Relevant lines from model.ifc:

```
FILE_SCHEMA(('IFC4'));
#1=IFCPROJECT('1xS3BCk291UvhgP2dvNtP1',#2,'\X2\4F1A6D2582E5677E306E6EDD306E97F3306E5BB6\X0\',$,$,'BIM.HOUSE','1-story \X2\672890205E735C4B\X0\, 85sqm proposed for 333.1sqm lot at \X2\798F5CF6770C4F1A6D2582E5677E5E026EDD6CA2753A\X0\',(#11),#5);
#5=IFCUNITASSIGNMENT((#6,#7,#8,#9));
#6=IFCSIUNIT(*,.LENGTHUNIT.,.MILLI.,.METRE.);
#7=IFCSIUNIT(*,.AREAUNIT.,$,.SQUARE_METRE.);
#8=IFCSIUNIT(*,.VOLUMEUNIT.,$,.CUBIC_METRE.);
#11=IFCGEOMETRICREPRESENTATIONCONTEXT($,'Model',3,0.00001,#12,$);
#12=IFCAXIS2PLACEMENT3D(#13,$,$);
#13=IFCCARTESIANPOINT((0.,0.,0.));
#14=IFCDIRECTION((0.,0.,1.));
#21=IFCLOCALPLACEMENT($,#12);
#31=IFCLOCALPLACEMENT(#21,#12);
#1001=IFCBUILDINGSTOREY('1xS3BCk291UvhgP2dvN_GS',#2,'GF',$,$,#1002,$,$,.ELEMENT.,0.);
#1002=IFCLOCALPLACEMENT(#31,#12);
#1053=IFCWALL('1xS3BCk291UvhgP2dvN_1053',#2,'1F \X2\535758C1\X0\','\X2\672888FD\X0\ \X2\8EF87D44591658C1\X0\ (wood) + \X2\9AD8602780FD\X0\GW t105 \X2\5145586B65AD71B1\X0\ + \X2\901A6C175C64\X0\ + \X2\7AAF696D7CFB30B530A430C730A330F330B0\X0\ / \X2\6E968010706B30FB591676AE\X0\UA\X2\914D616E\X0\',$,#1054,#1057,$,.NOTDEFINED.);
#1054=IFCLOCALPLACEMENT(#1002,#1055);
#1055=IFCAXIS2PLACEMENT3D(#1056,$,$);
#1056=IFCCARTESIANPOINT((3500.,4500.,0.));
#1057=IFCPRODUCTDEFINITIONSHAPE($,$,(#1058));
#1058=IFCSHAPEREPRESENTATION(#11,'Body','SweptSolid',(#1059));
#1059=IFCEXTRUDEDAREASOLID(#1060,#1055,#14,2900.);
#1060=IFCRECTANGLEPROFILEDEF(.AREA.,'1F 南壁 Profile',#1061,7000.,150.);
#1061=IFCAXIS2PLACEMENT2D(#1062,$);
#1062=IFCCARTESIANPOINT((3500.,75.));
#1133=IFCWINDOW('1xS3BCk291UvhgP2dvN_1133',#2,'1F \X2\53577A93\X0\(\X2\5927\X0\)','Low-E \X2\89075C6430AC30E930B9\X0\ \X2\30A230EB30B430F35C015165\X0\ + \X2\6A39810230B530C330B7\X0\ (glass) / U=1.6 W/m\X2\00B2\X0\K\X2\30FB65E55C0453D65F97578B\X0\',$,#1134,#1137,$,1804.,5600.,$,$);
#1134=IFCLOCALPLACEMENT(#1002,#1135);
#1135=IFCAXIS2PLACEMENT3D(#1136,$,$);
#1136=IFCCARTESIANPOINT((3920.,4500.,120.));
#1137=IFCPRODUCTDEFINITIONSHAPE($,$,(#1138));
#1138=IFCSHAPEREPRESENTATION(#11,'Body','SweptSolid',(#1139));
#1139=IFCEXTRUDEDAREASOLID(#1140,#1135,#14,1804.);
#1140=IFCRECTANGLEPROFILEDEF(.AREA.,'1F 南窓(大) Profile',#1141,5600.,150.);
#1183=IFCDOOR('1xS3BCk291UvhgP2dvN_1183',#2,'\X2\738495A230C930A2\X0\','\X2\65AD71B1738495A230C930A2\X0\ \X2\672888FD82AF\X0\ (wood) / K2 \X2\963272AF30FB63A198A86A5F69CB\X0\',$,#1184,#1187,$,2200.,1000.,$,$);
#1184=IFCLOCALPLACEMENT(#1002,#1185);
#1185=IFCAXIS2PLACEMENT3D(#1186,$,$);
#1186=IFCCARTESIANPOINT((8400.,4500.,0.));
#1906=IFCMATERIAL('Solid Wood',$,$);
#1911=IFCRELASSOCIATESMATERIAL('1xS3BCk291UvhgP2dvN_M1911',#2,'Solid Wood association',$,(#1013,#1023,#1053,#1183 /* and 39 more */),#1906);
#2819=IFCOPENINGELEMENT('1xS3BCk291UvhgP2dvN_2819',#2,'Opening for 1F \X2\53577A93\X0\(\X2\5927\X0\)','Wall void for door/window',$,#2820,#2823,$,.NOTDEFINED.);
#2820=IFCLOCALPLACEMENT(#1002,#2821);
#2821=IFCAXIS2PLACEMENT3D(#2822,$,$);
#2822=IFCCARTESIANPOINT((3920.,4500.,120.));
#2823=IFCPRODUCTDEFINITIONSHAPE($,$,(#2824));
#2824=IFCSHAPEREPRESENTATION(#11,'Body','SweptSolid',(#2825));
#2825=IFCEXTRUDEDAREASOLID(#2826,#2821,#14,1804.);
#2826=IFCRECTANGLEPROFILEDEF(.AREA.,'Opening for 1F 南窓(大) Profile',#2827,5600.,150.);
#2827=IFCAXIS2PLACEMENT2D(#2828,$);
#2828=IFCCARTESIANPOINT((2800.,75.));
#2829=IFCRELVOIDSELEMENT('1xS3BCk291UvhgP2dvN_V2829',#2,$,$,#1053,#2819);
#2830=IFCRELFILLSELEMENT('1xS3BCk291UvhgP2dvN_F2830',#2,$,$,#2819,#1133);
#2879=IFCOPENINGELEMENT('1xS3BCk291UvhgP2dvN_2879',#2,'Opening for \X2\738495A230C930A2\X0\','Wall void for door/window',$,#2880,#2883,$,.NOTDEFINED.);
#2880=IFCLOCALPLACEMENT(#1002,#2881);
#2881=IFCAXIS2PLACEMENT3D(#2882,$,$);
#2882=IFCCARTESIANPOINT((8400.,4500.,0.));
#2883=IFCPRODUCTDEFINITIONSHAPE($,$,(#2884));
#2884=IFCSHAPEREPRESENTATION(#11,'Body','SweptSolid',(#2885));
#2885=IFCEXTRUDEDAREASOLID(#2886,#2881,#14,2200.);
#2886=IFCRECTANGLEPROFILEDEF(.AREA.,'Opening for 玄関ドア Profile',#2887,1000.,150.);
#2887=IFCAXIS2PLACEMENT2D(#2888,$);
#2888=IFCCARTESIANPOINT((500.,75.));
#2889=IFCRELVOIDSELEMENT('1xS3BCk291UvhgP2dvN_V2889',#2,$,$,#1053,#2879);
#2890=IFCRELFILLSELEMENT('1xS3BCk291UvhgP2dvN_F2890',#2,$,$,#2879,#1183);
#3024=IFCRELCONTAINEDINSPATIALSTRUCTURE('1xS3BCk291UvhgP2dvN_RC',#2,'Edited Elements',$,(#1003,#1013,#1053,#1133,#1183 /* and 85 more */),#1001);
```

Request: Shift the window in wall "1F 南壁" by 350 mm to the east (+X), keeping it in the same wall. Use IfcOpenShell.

```python
import ifcopenshell
import ifcopenshell.api.geometry
import ifcopenshell.util.placement

model = ifcopenshell.open("model.ifc")

window = model.by_guid("1xS3BCk291UvhgP2dvN_1133")
opening = window.FillsVoids[0].RelatingOpeningElement
wall = opening.VoidsElements[0].RelatingBuildingElement

wall_matrix = ifcopenshell.util.placement.get_local_placement(wall.ObjectPlacement)
shift = wall_matrix[:3, 0] * 350.0
before = ifcopenshell.util.placement.get_local_placement(window.ObjectPlacement)[:3, 3].copy()

# The window is not placed relative to its opening, so move both.
for product in (opening, window):
    matrix = ifcopenshell.util.placement.get_local_placement(product.ObjectPlacement)
    matrix[:3, 3] += shift
    ifcopenshell.api.geometry.edit_object_placement(model, product=product, matrix=matrix, is_si=False)

after = ifcopenshell.util.placement.get_local_placement(window.ObjectPlacement)[:3, 3]
print("window moved by", (after - before).round(3) + 0.0)

model.write("model-out.ifc")
```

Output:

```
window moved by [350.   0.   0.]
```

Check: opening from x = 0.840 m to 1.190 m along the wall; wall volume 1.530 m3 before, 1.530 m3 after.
